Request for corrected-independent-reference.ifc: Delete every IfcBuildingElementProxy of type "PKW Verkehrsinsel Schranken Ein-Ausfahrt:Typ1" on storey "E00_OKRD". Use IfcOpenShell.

First a look at what the model holds.

```python
import ifcopenshell
import ifcopenshell.util.element

model = ifcopenshell.open("corrected-independent-reference.ifc")
print(model.schema)
storey = next(s for s in model.by_type("IfcBuildingStorey") if s.Name == "E00_OKRD")
proxies = [e for e in ifcopenshell.util.element.get_decomposition(storey) if e.is_a("IfcBuildingElementProxy")]
seen = {}
for e in proxies:
    element_type = ifcopenshell.util.element.get_type(e)
    name = element_type.Name if element_type not in (None, e) else None
    seen[name] = seen.get(name, 0) + 1
for name, count in sorted(seen.items(), key=str):
    print(count, "x", name)
```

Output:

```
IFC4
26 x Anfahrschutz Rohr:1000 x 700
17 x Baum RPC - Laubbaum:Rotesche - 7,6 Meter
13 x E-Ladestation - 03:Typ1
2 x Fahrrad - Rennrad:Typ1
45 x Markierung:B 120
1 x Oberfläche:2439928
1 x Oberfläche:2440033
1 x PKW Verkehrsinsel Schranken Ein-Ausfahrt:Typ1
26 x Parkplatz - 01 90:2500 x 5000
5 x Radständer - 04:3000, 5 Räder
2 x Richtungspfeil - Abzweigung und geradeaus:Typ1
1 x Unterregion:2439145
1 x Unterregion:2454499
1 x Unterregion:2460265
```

```python
import ifcopenshell
import ifcopenshell.api.root
import ifcopenshell.util.element

model = ifcopenshell.open("corrected-independent-reference.ifc")

storey = next(s for s in model.by_type("IfcBuildingStorey") if s.Name == "E00_OKRD")
proxies = [e for e in ifcopenshell.util.element.get_decomposition(storey) if e.is_a("IfcBuildingElementProxy")]
targets = [e for e in proxies if (t := ifcopenshell.util.element.get_type(e)) not in (None, e) and t.Name == "PKW Verkehrsinsel Schranken Ein-Ausfahrt:Typ1"]

for e in targets:
    ifcopenshell.api.root.remove_product(model, product=e)
print(len(targets), "removed")

model.write("corrected-independent-reference_rev.ifc")
```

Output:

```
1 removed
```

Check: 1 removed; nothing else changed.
